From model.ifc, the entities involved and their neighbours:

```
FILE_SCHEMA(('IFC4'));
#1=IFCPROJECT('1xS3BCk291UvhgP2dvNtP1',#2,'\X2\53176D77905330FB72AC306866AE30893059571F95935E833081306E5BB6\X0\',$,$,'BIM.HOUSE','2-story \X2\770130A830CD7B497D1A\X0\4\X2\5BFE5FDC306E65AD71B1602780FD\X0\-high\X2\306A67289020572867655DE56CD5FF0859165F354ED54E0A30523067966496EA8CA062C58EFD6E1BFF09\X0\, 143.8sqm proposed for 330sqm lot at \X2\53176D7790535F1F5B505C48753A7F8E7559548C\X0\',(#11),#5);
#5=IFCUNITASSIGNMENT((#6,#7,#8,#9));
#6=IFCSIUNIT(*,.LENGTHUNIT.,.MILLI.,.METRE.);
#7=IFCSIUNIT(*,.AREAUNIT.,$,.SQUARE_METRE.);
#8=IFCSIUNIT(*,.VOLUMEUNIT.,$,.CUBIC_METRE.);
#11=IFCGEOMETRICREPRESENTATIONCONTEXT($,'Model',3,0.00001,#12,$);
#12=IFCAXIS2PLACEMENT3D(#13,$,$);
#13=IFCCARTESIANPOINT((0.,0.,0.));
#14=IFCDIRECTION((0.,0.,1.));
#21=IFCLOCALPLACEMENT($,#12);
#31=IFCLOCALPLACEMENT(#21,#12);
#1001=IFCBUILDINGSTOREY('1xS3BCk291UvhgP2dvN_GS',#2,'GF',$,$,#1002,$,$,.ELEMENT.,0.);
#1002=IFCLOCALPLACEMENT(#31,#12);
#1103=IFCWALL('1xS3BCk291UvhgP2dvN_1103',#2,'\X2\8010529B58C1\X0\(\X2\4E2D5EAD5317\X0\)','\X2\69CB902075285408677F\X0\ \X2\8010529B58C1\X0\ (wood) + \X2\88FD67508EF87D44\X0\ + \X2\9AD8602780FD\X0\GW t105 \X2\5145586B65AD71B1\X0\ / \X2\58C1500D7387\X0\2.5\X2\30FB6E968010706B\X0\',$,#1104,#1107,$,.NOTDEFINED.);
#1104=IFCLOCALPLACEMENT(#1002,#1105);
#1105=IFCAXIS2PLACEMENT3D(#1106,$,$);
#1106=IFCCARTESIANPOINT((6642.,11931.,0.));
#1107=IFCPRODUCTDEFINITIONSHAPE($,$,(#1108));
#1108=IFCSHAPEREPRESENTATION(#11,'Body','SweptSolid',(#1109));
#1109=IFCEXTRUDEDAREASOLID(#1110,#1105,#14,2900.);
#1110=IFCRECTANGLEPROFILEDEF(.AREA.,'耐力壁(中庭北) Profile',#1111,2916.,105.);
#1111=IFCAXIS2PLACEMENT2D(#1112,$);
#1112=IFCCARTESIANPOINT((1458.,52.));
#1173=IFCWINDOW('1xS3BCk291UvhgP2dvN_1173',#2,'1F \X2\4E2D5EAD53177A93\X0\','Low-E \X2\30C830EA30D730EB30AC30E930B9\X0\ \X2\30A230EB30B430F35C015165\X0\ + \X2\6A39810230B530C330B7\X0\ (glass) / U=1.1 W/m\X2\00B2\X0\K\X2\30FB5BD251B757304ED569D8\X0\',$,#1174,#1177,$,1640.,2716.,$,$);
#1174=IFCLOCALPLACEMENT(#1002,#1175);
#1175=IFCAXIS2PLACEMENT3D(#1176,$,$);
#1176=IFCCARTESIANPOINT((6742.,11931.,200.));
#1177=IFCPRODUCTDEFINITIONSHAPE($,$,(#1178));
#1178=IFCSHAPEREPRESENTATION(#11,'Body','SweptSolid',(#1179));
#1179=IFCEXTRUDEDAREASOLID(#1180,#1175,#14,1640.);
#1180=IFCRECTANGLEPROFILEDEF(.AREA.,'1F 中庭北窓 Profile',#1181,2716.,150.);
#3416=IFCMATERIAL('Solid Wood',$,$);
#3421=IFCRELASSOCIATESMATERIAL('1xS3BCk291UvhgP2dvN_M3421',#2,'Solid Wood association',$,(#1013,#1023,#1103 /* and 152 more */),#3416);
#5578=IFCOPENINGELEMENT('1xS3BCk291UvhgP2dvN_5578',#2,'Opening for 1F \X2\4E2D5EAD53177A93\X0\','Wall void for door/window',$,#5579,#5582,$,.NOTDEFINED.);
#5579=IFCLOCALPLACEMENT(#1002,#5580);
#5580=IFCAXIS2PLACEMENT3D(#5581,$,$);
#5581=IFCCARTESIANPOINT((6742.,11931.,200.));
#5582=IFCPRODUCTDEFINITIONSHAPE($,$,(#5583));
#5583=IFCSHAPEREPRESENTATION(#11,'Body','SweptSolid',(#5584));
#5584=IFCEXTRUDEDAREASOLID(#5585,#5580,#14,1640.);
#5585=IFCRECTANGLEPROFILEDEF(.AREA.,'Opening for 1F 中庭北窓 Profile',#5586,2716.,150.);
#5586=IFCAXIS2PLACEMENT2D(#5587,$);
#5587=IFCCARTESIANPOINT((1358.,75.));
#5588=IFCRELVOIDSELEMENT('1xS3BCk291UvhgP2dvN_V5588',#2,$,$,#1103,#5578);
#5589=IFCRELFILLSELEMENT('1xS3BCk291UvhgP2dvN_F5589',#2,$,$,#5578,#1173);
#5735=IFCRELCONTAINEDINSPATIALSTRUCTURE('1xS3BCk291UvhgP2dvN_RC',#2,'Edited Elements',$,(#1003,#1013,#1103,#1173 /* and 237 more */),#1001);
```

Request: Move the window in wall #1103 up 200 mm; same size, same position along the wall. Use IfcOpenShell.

```python
import numpy as np
import ifcopenshell
import ifcopenshell.api.geometry
import ifcopenshell.util.placement
import ifcopenshell.util.unit

model = ifcopenshell.open("model.ifc")
unit_scale = ifcopenshell.util.unit.calculate_unit_scale(model)

window = model.by_guid("1xS3BCk291UvhgP2dvN_1173")
opening = window.FillsVoids[0].RelatingOpeningElement
dz = 0.2 / unit_scale

shift = np.array([0.0, 0.0, dz])
# The window is not placed relative to its opening, so move both.
for product in (opening, window):
    matrix = ifcopenshell.util.placement.get_local_placement(product.ObjectPlacement)
    matrix[:3, 3] += shift
    ifcopenshell.api.geometry.edit_object_placement(model, product=product, matrix=matrix, is_si=False)

print(f"moved by {dz * unit_scale:+.3f} m")

model.write("model_updated.ifc")
```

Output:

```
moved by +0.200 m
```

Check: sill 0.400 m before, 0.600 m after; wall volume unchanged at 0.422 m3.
